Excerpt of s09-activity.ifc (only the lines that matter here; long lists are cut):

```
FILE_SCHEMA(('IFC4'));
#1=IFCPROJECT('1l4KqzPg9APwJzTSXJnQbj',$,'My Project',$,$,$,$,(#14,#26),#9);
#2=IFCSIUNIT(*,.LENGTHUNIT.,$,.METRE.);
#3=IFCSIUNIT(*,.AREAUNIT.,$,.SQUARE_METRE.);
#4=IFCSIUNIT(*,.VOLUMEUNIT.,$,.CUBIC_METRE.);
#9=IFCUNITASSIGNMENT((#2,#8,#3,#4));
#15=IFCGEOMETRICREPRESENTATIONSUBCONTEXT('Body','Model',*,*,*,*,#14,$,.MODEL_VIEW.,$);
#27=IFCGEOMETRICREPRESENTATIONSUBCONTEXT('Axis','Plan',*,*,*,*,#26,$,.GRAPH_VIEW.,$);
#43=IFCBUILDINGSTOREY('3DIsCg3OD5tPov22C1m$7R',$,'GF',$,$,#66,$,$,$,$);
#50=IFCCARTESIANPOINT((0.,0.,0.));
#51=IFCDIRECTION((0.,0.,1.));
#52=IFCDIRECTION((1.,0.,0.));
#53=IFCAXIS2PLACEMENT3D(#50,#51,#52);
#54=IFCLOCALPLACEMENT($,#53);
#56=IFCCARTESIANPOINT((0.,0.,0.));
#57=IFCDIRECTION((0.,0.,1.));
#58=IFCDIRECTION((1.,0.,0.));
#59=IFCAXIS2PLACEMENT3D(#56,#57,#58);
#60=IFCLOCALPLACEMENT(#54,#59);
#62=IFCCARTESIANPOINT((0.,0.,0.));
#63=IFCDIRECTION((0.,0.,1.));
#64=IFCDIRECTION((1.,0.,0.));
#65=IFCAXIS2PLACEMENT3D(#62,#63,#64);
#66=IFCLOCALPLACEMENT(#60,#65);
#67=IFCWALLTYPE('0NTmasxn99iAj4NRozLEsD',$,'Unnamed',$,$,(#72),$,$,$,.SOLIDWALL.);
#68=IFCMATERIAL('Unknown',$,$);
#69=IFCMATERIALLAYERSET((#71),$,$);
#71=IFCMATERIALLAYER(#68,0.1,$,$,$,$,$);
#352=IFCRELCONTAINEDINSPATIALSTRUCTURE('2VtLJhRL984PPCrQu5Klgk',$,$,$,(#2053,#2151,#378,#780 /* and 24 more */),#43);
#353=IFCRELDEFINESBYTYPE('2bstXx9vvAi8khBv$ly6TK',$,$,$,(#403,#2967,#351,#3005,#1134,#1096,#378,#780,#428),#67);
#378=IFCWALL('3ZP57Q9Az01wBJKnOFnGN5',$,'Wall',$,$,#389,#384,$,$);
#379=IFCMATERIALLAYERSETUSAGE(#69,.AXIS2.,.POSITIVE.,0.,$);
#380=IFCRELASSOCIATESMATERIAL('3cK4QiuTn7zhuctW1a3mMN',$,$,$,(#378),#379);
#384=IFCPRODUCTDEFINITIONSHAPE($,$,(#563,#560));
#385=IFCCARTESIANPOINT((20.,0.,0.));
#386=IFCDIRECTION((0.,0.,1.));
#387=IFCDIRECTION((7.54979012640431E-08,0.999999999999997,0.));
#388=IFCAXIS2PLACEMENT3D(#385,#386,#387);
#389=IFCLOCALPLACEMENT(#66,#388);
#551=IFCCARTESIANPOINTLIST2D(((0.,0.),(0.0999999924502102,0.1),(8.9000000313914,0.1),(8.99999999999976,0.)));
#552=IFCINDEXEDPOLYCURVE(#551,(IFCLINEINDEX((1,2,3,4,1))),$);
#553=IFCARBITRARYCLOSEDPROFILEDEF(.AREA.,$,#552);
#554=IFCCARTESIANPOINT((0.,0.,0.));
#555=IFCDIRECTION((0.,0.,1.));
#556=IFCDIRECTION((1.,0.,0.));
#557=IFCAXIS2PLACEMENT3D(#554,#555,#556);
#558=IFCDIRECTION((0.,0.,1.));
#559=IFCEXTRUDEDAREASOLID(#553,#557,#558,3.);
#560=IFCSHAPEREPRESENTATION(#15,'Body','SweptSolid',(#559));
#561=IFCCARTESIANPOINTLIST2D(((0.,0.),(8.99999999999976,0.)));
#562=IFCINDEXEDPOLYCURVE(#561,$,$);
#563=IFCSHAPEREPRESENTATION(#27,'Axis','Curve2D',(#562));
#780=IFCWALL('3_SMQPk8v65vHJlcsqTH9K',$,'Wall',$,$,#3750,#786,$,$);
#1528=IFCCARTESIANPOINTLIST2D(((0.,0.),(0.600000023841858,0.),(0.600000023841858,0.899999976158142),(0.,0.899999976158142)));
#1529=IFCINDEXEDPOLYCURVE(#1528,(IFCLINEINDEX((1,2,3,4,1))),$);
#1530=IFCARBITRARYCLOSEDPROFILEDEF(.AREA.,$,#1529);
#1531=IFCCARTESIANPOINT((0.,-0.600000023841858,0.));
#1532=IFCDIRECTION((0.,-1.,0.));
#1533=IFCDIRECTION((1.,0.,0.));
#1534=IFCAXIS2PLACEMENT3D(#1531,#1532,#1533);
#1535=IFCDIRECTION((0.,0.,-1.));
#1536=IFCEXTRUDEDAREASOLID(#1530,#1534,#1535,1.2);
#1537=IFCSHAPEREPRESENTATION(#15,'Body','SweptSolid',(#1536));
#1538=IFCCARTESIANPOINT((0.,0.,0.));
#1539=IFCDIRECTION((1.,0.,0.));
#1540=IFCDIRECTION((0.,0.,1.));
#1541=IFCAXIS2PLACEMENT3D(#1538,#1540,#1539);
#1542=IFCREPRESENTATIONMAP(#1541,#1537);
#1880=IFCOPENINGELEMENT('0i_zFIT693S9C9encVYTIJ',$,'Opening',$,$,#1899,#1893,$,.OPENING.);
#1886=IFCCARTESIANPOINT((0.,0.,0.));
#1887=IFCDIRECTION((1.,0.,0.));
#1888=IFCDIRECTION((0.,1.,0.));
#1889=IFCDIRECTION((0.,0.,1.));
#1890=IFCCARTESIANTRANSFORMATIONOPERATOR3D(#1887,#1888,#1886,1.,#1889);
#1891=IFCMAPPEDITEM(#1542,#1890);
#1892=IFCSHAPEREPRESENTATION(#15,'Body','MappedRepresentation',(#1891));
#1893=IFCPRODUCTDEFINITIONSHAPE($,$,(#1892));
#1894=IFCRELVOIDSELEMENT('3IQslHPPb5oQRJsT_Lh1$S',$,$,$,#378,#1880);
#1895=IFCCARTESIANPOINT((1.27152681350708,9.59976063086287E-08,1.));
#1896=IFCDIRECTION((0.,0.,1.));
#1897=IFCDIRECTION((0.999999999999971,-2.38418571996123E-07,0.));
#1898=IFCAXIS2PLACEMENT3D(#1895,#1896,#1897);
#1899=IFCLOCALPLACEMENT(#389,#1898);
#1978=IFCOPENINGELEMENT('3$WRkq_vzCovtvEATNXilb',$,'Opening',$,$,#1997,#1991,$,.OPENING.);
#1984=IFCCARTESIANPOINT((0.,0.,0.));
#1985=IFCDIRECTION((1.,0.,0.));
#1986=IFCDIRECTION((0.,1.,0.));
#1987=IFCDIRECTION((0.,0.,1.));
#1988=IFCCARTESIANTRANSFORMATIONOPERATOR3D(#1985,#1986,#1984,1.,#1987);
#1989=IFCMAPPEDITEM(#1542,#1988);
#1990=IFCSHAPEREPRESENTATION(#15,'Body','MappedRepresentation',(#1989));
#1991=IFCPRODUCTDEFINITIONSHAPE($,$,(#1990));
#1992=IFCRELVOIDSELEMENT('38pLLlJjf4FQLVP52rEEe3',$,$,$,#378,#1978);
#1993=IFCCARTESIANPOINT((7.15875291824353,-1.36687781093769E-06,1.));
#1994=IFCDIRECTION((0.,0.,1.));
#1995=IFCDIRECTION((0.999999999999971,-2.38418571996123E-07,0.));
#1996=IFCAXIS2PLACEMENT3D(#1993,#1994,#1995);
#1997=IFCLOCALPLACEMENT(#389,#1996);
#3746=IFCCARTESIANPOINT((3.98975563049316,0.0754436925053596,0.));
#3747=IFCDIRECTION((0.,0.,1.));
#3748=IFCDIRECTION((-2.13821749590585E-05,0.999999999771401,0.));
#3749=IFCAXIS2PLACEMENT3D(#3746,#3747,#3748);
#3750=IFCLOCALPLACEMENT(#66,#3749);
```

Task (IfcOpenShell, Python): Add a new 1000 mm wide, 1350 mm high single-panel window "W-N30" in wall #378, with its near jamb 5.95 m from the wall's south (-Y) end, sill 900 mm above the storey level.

```python
import numpy as np
import ifcopenshell
import ifcopenshell.api.feature
import ifcopenshell.api.geometry
import ifcopenshell.api.root
import ifcopenshell.api.spatial
import ifcopenshell.geom
import ifcopenshell.util.element
import ifcopenshell.util.placement
import ifcopenshell.util.representation
import ifcopenshell.util.shape
import ifcopenshell.util.unit

model = ifcopenshell.open("s09-activity.ifc")
unit_scale = ifcopenshell.util.unit.calculate_unit_scale(model)
settings = ifcopenshell.geom.settings()


def volume(element):
    """Net volume in cubic metres, openings subtracted."""
    shape = ifcopenshell.geom.create_shape(settings, element)
    return ifcopenshell.util.shape.get_volume(shape.geometry)


wall = model.by_guid("3ZP57Q9Az01wBJKnOFnGN5")
storey = ifcopenshell.util.element.get_container(wall, ifc_class="IfcBuildingStorey")
context = ifcopenshell.util.representation.get_context(model, "Model", "Body", "MODEL_VIEW")
before = volume(wall)

width, height, from_end, sill = 1, 1.35, 5.95, 0.9  # metres

# The wall runs along its own X axis, and the end named is its -X end.
wall_shape = ifcopenshell.geom.create_shape(settings, wall)
x, y, z = ifcopenshell.util.shape.get_vertices(wall_shape.geometry).T
start = x.min() + from_end
face, thickness = float(y.min()), float(y.max() - y.min())
wall_matrix = ifcopenshell.util.placement.get_local_placement(wall.ObjectPlacement)
level = ifcopenshell.util.placement.get_local_placement(storey.ObjectPlacement)[2, 3]


def in_wall(x, y):
    """Placement at x, y metres in the wall's axes, at sill height."""
    matrix = wall_matrix.copy()
    matrix[:, 3] = wall_matrix @ np.array([x / unit_scale, y / unit_scale, 0.0, 1.0])
    matrix[2, 3] = level + sill / unit_scale
    return matrix


# Opening: a box that overshoots both wall faces by 50 mm.
opening = ifcopenshell.api.root.create_entity(model, ifc_class="IfcOpeningElement", predefined_type="OPENING")
box = ifcopenshell.api.geometry.add_wall_representation(
    model, context=context, length=width, height=height, thickness=thickness + 0.1
)
ifcopenshell.api.geometry.assign_representation(model, product=opening, representation=box)
ifcopenshell.api.geometry.edit_object_placement(model, product=opening, matrix=in_wall(start, face - 0.05), is_si=False)
ifcopenshell.api.feature.add_feature(model, feature=opening, element=wall)

window = ifcopenshell.api.root.create_entity(model, ifc_class="IfcWindow", name="W-N30", predefined_type="WINDOW")
window.OverallWidth, window.OverallHeight = width / unit_scale, height / unit_scale
window.PartitioningType = "SINGLE_PANEL"
body = ifcopenshell.api.geometry.add_window_representation(
    model,
    context=context,
    overall_width=window.OverallWidth,
    overall_height=window.OverallHeight,
    partition_type="SINGLE_PANEL",
)
ifcopenshell.api.geometry.assign_representation(model, product=window, representation=body)
ifcopenshell.api.spatial.assign_container(model, products=[window], relating_structure=storey)
ifcopenshell.api.feature.add_filling(model, opening=opening, element=window)

# Centre the window in the wall's thickness.
ifcopenshell.api.geometry.edit_object_placement(model, product=window, matrix=in_wall(start, face), is_si=False)
window_shape = ifcopenshell.geom.create_shape(settings, window)
depth = ifcopenshell.util.shape.get_vertices(window_shape.geometry)[:, 1]
offset = face + thickness / 2 - (depth.min() + depth.max()) / 2
ifcopenshell.api.geometry.edit_object_placement(model, product=window, matrix=in_wall(start, offset), is_si=False)

after = volume(wall)

print(f"wall volume {before:.3f} -> {after:.3f} m3")

model.write("s09-activity_v2.ifc")
```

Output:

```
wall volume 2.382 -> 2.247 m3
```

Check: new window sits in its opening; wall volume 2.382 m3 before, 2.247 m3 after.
